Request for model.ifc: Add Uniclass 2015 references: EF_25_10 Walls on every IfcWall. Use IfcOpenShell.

First a look at what the model holds.

```python
import ifcopenshell

model = ifcopenshell.open("model.ifc")
print(model.schema)
print("classifications:", [c.Name for c in model.by_type("IfcClassification")])
for ifc_class in ("IfcDoor", "IfcRoof", "IfcStair", "IfcWall", "IfcWindow"):
    print(ifc_class, len(model.by_type(ifc_class)))
```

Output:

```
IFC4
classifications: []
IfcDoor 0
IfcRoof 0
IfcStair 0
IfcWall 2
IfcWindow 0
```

```python
import ifcopenshell
import ifcopenshell.api.classification

model = ifcopenshell.open("model.ifc")

system = ifcopenshell.api.classification.add_classification(model, classification="Uniclass 2015")

codes = {
    "IfcWall": ("EF_25_10", "Walls"),
}
for ifc_class, (code, name) in codes.items():
    products = model.by_type(ifc_class)
    ifcopenshell.api.classification.add_reference(
        model, products=products, classification=system, identification=code, name=name
    )
    print(code, len(products))

model.write("model_v2.ifc")
```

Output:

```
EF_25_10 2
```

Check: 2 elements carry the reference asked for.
